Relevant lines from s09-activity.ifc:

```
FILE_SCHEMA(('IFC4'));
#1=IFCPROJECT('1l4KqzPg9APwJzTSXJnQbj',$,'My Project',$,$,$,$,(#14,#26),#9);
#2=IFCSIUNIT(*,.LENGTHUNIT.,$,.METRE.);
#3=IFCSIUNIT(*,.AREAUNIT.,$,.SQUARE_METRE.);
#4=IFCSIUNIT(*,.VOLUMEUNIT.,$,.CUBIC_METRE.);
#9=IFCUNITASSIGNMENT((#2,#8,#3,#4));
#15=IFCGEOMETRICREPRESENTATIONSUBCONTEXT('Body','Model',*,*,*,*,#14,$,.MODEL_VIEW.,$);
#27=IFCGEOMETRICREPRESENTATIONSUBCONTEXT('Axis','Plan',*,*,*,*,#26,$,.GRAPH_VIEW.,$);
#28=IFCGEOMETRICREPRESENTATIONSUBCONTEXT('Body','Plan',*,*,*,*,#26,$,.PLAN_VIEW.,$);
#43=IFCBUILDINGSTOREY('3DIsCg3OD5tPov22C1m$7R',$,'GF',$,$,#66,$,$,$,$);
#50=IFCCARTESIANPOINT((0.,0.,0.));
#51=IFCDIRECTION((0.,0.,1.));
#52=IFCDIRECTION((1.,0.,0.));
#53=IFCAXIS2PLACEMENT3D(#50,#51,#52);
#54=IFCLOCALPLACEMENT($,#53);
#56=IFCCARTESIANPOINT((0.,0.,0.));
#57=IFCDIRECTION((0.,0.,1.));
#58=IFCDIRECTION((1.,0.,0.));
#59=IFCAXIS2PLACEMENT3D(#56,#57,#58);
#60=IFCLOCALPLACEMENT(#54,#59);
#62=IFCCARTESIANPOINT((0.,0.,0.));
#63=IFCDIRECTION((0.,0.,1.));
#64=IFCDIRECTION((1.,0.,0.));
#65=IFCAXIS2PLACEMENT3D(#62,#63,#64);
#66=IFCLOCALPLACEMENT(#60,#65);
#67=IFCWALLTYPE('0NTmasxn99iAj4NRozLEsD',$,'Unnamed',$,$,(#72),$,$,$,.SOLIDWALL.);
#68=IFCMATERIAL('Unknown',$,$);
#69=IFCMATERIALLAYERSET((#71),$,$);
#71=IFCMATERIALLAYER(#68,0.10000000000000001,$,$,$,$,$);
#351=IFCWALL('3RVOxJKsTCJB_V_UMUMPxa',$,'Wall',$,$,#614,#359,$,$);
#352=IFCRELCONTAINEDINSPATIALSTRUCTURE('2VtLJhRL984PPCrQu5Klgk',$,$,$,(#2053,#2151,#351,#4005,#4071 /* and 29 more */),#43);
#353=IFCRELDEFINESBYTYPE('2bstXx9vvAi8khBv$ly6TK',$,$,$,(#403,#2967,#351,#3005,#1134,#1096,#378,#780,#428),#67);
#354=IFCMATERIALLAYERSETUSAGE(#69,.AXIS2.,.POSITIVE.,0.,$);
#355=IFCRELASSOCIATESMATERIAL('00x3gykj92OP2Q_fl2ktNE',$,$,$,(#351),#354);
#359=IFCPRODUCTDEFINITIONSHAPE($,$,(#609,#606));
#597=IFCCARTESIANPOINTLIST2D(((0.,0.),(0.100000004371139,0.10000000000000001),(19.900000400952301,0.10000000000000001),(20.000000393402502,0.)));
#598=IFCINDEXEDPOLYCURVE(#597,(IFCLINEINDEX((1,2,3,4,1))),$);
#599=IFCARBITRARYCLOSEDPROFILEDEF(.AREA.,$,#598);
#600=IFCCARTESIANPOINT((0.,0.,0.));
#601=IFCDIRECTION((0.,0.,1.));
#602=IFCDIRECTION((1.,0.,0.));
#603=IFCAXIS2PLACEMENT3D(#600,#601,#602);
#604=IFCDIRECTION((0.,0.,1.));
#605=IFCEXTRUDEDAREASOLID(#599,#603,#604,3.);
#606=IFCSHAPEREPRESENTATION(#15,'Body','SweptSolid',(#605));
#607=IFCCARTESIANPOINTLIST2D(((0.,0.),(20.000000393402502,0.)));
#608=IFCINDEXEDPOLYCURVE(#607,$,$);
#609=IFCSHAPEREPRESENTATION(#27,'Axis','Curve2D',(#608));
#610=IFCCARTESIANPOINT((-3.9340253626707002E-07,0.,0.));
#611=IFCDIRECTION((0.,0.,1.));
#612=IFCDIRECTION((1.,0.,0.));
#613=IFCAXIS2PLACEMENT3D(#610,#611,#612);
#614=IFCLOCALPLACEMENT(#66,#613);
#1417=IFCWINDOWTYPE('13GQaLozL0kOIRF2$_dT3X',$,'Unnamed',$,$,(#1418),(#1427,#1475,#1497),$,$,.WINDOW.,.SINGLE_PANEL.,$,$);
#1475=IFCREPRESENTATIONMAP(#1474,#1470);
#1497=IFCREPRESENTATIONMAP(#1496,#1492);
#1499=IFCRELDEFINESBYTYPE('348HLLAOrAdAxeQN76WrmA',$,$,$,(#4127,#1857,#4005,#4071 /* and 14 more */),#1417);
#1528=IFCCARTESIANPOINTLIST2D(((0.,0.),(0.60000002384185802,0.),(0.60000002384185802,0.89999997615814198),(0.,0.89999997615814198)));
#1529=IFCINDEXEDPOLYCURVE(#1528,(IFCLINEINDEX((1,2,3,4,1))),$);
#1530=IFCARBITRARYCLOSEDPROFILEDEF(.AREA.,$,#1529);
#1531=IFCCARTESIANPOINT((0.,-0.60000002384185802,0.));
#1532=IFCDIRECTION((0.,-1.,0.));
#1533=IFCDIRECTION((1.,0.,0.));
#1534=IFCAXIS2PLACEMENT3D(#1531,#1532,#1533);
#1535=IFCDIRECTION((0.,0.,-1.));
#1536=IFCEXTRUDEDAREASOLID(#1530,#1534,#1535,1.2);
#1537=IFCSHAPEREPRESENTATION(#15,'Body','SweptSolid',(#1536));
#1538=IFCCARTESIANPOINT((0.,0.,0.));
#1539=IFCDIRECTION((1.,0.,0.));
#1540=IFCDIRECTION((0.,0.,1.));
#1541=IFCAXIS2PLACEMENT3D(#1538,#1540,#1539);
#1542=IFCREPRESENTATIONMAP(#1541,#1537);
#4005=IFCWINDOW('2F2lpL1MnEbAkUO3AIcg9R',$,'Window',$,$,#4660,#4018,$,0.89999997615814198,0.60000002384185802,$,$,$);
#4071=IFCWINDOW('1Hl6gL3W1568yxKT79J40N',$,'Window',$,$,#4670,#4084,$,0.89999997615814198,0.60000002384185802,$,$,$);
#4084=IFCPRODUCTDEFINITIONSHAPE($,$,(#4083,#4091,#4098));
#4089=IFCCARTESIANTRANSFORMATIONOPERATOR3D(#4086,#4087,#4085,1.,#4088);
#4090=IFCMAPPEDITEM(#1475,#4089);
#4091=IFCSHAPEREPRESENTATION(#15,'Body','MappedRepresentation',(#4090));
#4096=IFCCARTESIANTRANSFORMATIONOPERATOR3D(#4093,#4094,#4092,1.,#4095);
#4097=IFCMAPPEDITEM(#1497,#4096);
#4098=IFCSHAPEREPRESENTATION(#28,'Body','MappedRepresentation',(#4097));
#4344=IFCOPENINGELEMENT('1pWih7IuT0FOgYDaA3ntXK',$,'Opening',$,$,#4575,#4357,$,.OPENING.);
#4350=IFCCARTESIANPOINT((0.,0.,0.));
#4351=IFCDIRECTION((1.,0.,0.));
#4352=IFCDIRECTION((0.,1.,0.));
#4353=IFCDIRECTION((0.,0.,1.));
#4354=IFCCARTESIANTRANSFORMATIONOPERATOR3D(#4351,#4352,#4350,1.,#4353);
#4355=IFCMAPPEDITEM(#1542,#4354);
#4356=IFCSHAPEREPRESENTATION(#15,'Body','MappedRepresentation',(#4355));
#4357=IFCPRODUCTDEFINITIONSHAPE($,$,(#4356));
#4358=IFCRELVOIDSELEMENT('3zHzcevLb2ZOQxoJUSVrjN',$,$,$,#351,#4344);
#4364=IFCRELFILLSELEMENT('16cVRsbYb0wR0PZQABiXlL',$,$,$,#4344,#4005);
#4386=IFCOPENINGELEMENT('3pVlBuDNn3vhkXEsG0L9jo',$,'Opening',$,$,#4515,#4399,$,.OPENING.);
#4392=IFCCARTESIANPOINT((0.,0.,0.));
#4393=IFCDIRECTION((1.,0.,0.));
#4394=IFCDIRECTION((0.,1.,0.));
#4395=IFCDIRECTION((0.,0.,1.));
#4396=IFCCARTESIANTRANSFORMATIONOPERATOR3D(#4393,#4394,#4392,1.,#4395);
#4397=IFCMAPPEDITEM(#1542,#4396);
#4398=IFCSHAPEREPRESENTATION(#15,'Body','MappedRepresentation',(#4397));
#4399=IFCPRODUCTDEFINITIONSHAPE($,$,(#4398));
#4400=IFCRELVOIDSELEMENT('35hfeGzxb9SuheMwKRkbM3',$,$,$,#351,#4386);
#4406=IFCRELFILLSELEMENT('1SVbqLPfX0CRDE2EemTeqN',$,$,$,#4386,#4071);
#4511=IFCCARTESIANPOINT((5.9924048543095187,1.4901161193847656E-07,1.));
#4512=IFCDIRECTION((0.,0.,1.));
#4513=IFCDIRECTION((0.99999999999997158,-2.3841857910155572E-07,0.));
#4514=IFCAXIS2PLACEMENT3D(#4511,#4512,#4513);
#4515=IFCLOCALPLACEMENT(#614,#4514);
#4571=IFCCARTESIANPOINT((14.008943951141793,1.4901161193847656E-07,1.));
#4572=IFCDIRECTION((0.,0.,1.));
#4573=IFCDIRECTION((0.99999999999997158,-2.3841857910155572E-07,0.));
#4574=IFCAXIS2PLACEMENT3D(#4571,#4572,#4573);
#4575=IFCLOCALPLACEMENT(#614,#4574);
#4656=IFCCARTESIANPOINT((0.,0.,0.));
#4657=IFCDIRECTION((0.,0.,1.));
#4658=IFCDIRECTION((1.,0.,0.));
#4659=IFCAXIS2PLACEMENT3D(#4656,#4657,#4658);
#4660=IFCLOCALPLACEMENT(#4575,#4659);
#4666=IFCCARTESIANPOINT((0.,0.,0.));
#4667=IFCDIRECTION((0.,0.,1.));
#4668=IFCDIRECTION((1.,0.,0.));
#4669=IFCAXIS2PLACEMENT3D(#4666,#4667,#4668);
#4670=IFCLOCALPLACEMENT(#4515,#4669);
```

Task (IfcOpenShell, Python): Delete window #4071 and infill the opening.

```python
import ifcopenshell
import ifcopenshell.api.feature
import ifcopenshell.api.root
import ifcopenshell.geom
import ifcopenshell.util.shape

model = ifcopenshell.open("s09-activity.ifc")
settings = ifcopenshell.geom.settings()


def volume(element):
    """Net volume in cubic metres, openings subtracted."""
    shape = ifcopenshell.geom.create_shape(settings, element)
    return ifcopenshell.util.shape.get_volume(shape.geometry)


window = model.by_id(4071)
opening = window.FillsVoids[0].RelatingOpeningElement
wall = opening.VoidsElements[0].RelatingBuildingElement
before = volume(wall)

ifcopenshell.api.root.remove_product(model, product=window)
ifcopenshell.api.feature.remove_feature(model, feature=opening)

after = volume(wall)

print(f"wall volume {before:.3f} -> {after:.3f} m3")

model.write("s09-activity_updated.ifc")
```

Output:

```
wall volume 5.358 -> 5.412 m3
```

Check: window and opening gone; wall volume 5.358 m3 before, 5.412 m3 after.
